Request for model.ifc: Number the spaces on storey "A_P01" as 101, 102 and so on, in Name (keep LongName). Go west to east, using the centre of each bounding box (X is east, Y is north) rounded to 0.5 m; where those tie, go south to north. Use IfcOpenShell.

First a look at what the model holds.

```python
import ifcopenshell
import ifcopenshell.util.element
import ifcopenshell.util.placement

model = ifcopenshell.open("model.ifc")
print(model.schema)
storey = next(s for s in model.by_type("IfcBuildingStorey") if s.Name == "A_P01")
spaces = [e for e in ifcopenshell.util.element.get_decomposition(storey) if e.is_a("IfcSpace")]
for e in sorted(spaces, key=lambda e: e.id()):
    origin = ifcopenshell.util.placement.get_local_placement(e.ObjectPlacement)[:3, 3]
    print(e.id(), e.Name, e.LongName, origin.round(2) + 0.0, sep=" | ")
```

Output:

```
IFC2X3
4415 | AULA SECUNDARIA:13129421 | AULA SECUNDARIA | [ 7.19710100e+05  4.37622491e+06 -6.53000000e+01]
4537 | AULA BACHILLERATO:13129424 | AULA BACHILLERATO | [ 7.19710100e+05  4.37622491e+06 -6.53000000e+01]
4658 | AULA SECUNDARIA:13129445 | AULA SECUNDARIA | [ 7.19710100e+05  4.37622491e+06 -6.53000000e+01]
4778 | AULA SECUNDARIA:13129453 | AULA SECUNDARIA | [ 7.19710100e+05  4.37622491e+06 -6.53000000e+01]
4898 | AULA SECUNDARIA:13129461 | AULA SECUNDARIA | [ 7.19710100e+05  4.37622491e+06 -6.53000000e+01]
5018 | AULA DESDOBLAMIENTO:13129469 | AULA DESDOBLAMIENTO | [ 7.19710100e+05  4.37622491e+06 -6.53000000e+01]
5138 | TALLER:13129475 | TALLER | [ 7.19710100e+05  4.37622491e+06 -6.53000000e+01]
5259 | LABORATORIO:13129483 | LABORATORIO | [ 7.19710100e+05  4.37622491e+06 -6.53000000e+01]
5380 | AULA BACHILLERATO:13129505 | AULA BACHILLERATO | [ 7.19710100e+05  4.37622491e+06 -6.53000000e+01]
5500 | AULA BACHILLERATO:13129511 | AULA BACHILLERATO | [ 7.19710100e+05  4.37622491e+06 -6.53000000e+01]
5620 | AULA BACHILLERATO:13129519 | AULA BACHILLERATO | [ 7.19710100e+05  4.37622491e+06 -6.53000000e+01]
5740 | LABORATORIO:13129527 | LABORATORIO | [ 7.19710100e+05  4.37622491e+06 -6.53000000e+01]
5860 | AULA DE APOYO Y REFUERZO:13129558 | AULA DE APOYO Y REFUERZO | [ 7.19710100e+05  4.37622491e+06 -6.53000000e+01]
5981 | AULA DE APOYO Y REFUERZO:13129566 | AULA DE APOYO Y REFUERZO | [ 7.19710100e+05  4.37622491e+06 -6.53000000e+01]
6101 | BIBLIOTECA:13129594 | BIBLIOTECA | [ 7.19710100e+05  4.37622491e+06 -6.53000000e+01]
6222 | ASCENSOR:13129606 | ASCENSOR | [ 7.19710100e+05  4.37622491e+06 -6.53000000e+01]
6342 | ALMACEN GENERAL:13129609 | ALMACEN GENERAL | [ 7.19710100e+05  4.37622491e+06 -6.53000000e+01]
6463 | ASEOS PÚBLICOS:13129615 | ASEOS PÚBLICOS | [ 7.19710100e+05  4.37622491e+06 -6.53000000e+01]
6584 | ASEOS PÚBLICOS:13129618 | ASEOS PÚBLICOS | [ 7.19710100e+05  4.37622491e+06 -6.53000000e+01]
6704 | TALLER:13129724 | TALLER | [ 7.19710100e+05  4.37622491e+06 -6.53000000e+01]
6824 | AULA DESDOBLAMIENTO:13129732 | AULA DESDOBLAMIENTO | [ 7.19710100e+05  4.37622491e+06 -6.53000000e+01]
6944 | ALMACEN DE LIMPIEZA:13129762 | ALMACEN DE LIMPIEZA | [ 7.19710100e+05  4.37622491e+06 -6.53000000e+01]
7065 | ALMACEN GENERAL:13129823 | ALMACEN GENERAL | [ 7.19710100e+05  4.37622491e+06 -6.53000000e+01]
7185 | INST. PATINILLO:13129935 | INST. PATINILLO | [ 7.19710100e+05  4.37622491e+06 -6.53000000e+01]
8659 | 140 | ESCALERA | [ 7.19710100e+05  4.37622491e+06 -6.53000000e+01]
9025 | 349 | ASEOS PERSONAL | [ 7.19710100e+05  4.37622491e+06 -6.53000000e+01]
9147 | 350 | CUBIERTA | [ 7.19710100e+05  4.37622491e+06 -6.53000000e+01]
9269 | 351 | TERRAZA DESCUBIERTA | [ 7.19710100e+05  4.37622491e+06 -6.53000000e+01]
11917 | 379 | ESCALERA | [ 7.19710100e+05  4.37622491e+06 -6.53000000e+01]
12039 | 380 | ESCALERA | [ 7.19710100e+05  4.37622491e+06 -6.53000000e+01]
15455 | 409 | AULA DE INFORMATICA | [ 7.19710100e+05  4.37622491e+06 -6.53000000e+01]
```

```python
import ifcopenshell
import ifcopenshell.geom
import ifcopenshell.util.element
import ifcopenshell.util.shape

model = ifcopenshell.open("model.ifc")
settings = ifcopenshell.geom.settings()
settings.set("use-world-coords", True)


def centre(element):
    shape = ifcopenshell.geom.create_shape(settings, element)
    return ifcopenshell.util.shape.get_bbox_centroid(shape.geometry)


storey = next(s for s in model.by_type("IfcBuildingStorey") if s.Name == "A_P01")
spaces = [e for e in ifcopenshell.util.element.get_decomposition(storey) if e.is_a("IfcSpace")]

# Insertion points can sit at a corner or the storey origin, so sort by the geometry (in metres).
centres = {e: centre(e) for e in spaces}
spaces.sort(key=lambda e: (round(centres[e][0] / 0.5), centres[e][1]))

for i, e in enumerate(spaces, start=1):
    number = f"1{i:02d}"
    e.Name = number
    print(e.id(), number)

model.write("model_updated.ifc")
```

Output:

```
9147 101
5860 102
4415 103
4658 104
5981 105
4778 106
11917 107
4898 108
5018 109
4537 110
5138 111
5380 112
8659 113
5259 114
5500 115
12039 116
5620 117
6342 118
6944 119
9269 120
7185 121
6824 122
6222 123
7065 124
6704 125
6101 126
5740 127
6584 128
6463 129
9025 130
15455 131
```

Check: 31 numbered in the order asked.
